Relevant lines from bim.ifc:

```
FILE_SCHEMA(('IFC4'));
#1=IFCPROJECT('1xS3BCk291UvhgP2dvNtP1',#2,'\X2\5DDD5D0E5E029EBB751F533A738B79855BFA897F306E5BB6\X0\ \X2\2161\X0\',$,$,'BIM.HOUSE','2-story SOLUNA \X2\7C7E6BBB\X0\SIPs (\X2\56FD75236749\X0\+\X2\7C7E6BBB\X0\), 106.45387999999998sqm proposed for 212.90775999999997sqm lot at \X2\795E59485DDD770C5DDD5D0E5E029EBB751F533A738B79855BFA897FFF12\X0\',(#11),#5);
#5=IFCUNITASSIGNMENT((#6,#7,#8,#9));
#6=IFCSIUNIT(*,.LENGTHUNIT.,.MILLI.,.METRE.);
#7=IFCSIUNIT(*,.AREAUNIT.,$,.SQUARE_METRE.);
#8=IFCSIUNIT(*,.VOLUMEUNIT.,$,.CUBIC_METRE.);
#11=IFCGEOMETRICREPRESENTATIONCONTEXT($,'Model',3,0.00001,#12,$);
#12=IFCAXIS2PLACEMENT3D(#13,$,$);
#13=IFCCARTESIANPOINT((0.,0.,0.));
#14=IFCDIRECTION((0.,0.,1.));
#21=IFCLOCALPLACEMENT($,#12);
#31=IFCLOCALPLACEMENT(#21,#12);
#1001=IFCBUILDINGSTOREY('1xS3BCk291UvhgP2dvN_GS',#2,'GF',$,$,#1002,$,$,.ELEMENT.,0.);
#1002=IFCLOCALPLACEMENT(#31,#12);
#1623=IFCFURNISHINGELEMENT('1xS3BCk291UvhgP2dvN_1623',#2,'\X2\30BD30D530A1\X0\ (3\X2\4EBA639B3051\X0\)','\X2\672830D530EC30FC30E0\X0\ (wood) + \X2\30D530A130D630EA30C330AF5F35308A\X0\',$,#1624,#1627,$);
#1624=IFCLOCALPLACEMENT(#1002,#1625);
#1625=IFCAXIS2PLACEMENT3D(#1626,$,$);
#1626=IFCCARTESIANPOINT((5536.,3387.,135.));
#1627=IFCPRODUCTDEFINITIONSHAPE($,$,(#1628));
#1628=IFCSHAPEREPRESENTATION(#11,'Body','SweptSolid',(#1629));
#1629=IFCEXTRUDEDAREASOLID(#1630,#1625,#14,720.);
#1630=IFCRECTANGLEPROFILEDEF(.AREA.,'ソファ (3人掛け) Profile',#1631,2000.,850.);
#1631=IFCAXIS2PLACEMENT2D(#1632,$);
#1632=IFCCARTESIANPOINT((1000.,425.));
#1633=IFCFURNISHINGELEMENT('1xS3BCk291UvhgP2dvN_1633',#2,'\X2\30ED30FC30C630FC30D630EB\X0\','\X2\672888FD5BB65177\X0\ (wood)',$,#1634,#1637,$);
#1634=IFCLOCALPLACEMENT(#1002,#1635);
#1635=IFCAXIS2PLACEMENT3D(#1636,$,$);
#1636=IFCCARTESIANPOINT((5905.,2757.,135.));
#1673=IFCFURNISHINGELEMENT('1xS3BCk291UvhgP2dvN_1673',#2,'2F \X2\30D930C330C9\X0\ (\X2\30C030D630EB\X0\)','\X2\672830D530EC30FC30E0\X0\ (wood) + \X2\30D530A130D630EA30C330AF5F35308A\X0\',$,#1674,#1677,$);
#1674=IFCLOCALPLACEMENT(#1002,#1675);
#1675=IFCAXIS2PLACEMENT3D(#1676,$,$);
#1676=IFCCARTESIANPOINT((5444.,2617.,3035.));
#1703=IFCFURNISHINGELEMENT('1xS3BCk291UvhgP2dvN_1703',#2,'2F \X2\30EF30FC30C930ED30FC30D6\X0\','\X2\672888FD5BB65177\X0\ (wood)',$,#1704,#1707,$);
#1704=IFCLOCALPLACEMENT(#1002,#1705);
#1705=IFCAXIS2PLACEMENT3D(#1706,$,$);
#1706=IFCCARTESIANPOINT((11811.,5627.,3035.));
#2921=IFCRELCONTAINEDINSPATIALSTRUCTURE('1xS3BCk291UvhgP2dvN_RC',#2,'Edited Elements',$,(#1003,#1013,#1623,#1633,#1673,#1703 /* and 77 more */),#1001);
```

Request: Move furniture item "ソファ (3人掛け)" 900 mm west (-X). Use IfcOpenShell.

```python
import ifcopenshell
import ifcopenshell.api.geometry
import ifcopenshell.util.placement
import ifcopenshell.util.unit

model = ifcopenshell.open("bim.ifc")
unit_scale = ifcopenshell.util.unit.calculate_unit_scale(model)

item = model.by_guid("1xS3BCk291UvhgP2dvN_1623")
matrix = ifcopenshell.util.placement.get_local_placement(item.ObjectPlacement)
matrix[0, 3] -= 0.9 / unit_scale
ifcopenshell.api.geometry.edit_object_placement(model, product=item, matrix=matrix, is_si=False)

print(ifcopenshell.util.placement.get_local_placement(item.ObjectPlacement).round(3) + 0.0)

model.write("bim_edited.ifc")
```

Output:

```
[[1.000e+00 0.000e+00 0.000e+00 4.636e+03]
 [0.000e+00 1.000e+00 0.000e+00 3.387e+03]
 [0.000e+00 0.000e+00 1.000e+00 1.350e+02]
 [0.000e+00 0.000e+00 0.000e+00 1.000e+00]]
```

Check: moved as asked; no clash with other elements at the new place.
